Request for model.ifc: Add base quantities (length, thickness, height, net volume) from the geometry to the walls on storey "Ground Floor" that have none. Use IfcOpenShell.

First a look at what the model holds.

```python
import ifcopenshell
import ifcopenshell.util.element
import ifcopenshell.util.unit

model = ifcopenshell.open("model.ifc")
print(model.schema)
for unit_type in ("LENGTHUNIT", "AREAUNIT", "VOLUMEUNIT"):
    print(unit_type, ifcopenshell.util.unit.calculate_unit_scale(model, unit_type))
storey = next(s for s in model.by_type("IfcBuildingStorey") if s.Name == "Ground Floor")
walls = [e for e in ifcopenshell.util.element.get_decomposition(storey) if e.is_a("IfcWall")]
for e in sorted(walls, key=lambda e: e.id()):
    print(e.id(), e.is_a(), e.Name, list(ifcopenshell.util.element.get_psets(e, qtos_only=True)), sep=" | ")
```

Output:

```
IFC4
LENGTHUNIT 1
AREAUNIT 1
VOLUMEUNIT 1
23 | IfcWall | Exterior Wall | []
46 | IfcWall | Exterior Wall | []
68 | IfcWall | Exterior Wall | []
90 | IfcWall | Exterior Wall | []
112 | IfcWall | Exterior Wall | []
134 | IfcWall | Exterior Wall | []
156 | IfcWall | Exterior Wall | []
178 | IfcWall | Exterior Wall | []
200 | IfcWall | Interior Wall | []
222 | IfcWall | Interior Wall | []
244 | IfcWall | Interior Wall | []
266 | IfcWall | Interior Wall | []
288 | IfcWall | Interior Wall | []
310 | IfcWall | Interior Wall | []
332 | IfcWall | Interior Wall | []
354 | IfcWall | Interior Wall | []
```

```python
import ifcopenshell
import ifcopenshell.api.pset
import ifcopenshell.geom
import ifcopenshell.util.element
import ifcopenshell.util.shape
import ifcopenshell.util.unit

model = ifcopenshell.open("model.ifc")
unit_scale = ifcopenshell.util.unit.calculate_unit_scale(model)
volume_scale = ifcopenshell.util.unit.calculate_unit_scale(model, "VOLUMEUNIT")
settings = ifcopenshell.geom.settings()

storey = next(s for s in model.by_type("IfcBuildingStorey") if s.Name == "Ground Floor")
walls = [e for e in ifcopenshell.util.element.get_decomposition(storey) if e.is_a("IfcWall")]

for e in sorted(walls, key=lambda e: e.id()):
    if ifcopenshell.util.element.get_psets(e, qtos_only=True, should_inherit=False):
        continue
    # Geometry comes back in metres, in the element's own axes.
    shape = ifcopenshell.geom.create_shape(settings, e)
    values = {
        "Length": ifcopenshell.util.shape.get_x(shape.geometry) / unit_scale,
        "Width": ifcopenshell.util.shape.get_y(shape.geometry) / unit_scale,
        "Height": ifcopenshell.util.shape.get_z(shape.geometry) / unit_scale,
        "NetVolume": ifcopenshell.util.shape.get_volume(shape.geometry) / volume_scale,
    }
    qto = ifcopenshell.api.pset.add_qto(model, product=e, name="Qto_WallBaseQuantities")
    ifcopenshell.api.pset.edit_qto(model, qto=qto, properties=values)
    print(e.id(), {k: round(v, 3) for k, v in values.items()})

model.write("model_v2.ifc")
```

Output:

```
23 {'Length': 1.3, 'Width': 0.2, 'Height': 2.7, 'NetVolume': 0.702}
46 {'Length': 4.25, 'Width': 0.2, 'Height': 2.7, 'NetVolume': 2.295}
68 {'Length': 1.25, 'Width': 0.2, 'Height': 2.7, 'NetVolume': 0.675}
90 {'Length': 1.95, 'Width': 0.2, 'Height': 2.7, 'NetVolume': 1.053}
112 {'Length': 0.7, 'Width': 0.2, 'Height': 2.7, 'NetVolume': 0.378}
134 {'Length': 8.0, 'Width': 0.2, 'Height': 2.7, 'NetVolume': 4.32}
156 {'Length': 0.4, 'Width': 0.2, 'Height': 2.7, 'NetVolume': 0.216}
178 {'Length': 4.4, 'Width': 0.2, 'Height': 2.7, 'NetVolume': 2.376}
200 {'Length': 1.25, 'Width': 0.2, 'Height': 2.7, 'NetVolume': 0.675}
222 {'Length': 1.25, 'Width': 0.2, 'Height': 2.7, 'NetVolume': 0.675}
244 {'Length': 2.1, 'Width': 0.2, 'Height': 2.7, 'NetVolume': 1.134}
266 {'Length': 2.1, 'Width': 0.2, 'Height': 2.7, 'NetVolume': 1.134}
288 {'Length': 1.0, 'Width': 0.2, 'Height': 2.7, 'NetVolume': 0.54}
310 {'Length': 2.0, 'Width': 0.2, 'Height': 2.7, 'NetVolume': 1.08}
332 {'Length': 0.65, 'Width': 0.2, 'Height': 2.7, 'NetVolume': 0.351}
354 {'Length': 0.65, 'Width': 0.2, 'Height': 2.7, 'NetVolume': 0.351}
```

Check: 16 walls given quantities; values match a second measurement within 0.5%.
